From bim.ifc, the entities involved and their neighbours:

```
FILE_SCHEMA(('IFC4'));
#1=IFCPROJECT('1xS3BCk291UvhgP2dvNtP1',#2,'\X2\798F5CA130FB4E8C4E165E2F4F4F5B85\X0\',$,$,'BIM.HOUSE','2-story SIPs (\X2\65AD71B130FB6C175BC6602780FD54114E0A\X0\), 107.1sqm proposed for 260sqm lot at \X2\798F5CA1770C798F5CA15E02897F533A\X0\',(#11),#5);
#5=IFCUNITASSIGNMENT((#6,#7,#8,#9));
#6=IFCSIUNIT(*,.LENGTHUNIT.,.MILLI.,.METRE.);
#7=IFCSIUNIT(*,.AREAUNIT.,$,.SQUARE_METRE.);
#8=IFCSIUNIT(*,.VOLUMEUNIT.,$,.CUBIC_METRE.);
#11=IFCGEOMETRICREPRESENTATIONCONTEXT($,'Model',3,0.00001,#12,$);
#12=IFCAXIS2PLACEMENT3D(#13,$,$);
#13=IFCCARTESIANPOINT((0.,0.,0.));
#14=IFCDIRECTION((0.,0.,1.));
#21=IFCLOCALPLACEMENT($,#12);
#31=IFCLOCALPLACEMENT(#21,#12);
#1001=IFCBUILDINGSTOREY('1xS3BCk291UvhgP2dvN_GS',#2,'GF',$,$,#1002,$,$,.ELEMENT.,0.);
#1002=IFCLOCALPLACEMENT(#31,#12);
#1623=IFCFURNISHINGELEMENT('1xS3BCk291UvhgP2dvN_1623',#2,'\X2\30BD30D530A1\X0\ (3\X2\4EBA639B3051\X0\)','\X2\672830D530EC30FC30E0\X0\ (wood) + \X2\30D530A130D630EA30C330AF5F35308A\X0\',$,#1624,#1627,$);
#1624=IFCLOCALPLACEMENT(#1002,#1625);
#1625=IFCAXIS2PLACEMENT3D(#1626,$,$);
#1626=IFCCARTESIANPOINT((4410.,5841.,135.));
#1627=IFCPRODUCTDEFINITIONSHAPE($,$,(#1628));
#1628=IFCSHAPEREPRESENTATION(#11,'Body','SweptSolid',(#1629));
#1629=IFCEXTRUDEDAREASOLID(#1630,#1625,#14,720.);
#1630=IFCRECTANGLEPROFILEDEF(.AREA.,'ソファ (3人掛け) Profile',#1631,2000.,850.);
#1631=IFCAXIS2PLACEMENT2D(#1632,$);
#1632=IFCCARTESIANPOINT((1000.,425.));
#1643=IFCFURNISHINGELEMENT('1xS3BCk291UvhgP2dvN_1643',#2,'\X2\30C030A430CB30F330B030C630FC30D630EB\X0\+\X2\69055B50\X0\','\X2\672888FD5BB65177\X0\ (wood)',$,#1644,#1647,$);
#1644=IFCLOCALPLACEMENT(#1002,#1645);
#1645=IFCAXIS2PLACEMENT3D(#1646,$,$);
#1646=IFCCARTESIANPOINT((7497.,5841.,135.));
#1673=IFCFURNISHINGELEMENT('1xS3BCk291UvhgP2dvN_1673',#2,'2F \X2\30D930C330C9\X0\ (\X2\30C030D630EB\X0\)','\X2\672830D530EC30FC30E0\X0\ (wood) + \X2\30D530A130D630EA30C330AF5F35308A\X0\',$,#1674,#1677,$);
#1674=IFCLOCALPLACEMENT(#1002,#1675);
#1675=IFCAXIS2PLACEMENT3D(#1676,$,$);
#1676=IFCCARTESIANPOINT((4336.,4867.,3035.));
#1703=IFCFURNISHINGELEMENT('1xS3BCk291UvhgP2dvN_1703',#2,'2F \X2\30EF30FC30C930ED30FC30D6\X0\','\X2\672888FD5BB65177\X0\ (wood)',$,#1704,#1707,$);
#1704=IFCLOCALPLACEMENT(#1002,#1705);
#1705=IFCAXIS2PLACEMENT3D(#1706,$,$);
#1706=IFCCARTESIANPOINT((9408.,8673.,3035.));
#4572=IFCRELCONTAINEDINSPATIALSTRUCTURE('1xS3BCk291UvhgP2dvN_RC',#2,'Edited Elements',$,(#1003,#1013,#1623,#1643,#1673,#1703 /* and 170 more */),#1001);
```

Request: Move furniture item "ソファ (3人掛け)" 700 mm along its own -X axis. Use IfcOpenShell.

```python
import ifcopenshell
import ifcopenshell.api.geometry
import ifcopenshell.util.placement
import ifcopenshell.util.unit

model = ifcopenshell.open("bim.ifc")
unit_scale = ifcopenshell.util.unit.calculate_unit_scale(model)

item = model.by_guid("1xS3BCk291UvhgP2dvN_1623")
matrix = ifcopenshell.util.placement.get_local_placement(item.ObjectPlacement)
matrix[:3, 3] -= matrix[:3, 0] * 0.7 / unit_scale
ifcopenshell.api.geometry.edit_object_placement(model, product=item, matrix=matrix, is_si=False)

print(ifcopenshell.util.placement.get_local_placement(item.ObjectPlacement).round(3) + 0.0)

model.write("bim_rev.ifc")
```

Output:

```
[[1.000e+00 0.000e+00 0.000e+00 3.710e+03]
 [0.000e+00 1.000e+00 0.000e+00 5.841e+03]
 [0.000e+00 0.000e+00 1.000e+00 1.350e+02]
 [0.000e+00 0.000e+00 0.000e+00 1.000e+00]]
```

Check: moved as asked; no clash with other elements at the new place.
